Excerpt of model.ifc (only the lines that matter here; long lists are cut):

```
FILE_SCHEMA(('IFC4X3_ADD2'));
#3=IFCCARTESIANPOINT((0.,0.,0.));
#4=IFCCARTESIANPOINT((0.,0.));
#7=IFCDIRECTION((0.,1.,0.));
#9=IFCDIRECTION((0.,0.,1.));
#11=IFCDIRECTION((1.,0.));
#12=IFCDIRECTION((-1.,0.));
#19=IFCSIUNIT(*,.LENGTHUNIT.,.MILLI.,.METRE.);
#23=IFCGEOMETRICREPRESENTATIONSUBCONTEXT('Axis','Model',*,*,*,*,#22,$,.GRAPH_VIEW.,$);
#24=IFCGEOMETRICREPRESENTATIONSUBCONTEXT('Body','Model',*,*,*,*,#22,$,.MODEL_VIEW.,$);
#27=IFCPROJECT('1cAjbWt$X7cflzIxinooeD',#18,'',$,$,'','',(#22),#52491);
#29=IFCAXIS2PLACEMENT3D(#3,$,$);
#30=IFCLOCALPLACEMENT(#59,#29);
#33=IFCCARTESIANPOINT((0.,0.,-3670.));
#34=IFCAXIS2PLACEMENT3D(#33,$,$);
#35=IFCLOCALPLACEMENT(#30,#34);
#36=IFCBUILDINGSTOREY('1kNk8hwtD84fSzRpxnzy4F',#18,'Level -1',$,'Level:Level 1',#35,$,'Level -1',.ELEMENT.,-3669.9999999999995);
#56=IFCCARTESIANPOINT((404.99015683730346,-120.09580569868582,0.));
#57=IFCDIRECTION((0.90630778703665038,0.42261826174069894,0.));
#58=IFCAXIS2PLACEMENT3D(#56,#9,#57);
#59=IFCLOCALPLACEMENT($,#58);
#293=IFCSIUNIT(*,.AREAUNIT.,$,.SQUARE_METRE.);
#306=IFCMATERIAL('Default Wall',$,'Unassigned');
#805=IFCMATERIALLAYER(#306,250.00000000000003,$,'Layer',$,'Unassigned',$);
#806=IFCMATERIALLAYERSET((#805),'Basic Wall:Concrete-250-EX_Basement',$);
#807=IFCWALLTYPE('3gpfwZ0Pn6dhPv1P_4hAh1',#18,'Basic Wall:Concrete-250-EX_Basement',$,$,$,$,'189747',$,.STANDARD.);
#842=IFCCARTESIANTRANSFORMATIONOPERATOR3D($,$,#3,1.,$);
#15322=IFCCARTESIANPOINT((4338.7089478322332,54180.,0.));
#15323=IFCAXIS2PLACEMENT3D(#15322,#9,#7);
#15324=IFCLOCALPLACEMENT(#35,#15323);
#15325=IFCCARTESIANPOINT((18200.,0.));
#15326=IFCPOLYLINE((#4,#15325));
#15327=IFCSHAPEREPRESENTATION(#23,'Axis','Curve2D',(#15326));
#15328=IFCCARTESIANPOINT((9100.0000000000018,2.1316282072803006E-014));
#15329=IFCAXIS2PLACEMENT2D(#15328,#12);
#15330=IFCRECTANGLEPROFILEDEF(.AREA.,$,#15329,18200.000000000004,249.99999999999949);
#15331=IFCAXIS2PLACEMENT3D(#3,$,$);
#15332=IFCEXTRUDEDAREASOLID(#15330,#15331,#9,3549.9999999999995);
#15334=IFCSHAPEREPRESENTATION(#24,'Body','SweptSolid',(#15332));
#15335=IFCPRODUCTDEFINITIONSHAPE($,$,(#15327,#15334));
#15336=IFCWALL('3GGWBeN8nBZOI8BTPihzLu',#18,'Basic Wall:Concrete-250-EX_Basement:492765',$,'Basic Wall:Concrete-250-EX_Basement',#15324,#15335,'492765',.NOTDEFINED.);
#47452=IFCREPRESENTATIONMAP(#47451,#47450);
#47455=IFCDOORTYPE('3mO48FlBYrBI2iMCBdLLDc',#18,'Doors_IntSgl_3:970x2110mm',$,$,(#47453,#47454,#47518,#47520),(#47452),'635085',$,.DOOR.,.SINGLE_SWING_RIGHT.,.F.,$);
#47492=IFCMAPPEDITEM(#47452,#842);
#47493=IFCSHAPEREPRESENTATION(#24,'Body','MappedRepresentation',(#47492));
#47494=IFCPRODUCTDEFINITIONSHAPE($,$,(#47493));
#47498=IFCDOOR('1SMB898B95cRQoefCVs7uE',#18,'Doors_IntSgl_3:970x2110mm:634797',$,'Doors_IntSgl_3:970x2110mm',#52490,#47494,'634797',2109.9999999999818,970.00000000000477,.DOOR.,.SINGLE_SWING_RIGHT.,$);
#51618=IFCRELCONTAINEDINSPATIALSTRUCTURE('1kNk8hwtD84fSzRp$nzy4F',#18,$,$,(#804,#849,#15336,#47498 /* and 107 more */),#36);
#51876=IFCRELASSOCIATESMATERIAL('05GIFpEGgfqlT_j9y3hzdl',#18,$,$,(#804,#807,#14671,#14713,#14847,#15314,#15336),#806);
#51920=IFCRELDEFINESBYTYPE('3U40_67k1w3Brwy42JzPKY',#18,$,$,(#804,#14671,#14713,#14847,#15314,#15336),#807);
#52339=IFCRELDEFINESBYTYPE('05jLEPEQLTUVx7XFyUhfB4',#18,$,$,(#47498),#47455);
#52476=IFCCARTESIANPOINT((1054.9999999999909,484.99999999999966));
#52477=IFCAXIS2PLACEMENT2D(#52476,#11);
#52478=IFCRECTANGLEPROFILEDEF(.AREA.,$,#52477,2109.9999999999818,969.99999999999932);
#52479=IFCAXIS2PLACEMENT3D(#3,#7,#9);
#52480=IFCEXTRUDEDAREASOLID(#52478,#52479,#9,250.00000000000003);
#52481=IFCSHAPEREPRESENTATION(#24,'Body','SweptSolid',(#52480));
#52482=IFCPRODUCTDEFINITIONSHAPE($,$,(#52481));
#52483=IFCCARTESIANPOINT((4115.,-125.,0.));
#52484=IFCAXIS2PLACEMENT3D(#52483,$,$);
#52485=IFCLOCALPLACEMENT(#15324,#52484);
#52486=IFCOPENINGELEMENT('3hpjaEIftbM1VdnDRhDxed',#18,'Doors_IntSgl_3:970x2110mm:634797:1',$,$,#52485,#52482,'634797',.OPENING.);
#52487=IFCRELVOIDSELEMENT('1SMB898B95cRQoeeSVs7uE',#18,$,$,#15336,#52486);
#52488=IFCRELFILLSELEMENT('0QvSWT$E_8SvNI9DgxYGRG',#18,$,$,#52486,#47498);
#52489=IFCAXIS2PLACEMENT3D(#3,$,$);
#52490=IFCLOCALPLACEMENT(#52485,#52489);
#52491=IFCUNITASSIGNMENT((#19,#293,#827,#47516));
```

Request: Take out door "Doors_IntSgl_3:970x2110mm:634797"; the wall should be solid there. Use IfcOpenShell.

```python
import ifcopenshell
import ifcopenshell.api.feature
import ifcopenshell.api.root
import ifcopenshell.geom
import ifcopenshell.util.shape

model = ifcopenshell.open("model.ifc")
settings = ifcopenshell.geom.settings()


def volume(element):
    """Net volume in cubic metres, openings subtracted."""
    shape = ifcopenshell.geom.create_shape(settings, element)
    return ifcopenshell.util.shape.get_volume(shape.geometry)


door = model.by_guid("1SMB898B95cRQoefCVs7uE")
opening = door.FillsVoids[0].RelatingOpeningElement
wall = opening.VoidsElements[0].RelatingBuildingElement
before = volume(wall)

ifcopenshell.api.root.remove_product(model, product=door)
ifcopenshell.api.feature.remove_feature(model, feature=opening)

after = volume(wall)

print(f"wall volume {before:.3f} -> {after:.3f} m3")

model.write("model-out.ifc")
```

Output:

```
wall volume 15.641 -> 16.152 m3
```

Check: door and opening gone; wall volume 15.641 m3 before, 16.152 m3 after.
